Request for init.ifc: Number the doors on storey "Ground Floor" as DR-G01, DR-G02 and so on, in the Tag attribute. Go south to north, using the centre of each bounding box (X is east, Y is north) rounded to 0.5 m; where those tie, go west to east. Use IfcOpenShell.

First a look at what the model holds.

```python
import ifcopenshell
import ifcopenshell.util.element
import ifcopenshell.util.placement

model = ifcopenshell.open("init.ifc")
print(model.schema)
storey = next(s for s in model.by_type("IfcBuildingStorey") if s.Name == "Ground Floor")
doors = [e for e in ifcopenshell.util.element.get_decomposition(storey) if e.is_a("IfcDoor")]
for e in sorted(doors, key=lambda e: e.id()):
    origin = ifcopenshell.util.placement.get_local_placement(e.ObjectPlacement)[:3, 3]
    print(e.id(), e.Tag, e.Name, origin.round(2) + 0.0, sep=" | ")
```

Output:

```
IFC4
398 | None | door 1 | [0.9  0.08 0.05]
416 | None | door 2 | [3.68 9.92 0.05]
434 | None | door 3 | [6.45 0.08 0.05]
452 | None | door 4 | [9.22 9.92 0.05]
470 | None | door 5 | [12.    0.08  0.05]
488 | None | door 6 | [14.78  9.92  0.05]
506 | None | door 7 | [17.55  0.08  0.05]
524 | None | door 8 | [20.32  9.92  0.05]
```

```python
import ifcopenshell
import ifcopenshell.geom
import ifcopenshell.util.element
import ifcopenshell.util.shape

model = ifcopenshell.open("init.ifc")
settings = ifcopenshell.geom.settings()
settings.set("use-world-coords", True)


def centre(element):
    shape = ifcopenshell.geom.create_shape(settings, element)
    return ifcopenshell.util.shape.get_bbox_centroid(shape.geometry)


storey = next(s for s in model.by_type("IfcBuildingStorey") if s.Name == "Ground Floor")
doors = [e for e in ifcopenshell.util.element.get_decomposition(storey) if e.is_a("IfcDoor")]

# Insertion points can sit at a corner or the storey origin, so sort by the geometry (in metres).
centres = {e: centre(e) for e in doors}
doors.sort(key=lambda e: (round(centres[e][1] / 0.5), centres[e][0]))

for i, e in enumerate(doors, start=1):
    number = f"DR-G{i:02d}"
    e.Tag = number
    print(e.id(), number)

model.write("init_rev.ifc")
```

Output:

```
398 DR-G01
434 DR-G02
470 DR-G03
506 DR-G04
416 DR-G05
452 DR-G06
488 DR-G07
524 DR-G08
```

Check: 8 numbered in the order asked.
